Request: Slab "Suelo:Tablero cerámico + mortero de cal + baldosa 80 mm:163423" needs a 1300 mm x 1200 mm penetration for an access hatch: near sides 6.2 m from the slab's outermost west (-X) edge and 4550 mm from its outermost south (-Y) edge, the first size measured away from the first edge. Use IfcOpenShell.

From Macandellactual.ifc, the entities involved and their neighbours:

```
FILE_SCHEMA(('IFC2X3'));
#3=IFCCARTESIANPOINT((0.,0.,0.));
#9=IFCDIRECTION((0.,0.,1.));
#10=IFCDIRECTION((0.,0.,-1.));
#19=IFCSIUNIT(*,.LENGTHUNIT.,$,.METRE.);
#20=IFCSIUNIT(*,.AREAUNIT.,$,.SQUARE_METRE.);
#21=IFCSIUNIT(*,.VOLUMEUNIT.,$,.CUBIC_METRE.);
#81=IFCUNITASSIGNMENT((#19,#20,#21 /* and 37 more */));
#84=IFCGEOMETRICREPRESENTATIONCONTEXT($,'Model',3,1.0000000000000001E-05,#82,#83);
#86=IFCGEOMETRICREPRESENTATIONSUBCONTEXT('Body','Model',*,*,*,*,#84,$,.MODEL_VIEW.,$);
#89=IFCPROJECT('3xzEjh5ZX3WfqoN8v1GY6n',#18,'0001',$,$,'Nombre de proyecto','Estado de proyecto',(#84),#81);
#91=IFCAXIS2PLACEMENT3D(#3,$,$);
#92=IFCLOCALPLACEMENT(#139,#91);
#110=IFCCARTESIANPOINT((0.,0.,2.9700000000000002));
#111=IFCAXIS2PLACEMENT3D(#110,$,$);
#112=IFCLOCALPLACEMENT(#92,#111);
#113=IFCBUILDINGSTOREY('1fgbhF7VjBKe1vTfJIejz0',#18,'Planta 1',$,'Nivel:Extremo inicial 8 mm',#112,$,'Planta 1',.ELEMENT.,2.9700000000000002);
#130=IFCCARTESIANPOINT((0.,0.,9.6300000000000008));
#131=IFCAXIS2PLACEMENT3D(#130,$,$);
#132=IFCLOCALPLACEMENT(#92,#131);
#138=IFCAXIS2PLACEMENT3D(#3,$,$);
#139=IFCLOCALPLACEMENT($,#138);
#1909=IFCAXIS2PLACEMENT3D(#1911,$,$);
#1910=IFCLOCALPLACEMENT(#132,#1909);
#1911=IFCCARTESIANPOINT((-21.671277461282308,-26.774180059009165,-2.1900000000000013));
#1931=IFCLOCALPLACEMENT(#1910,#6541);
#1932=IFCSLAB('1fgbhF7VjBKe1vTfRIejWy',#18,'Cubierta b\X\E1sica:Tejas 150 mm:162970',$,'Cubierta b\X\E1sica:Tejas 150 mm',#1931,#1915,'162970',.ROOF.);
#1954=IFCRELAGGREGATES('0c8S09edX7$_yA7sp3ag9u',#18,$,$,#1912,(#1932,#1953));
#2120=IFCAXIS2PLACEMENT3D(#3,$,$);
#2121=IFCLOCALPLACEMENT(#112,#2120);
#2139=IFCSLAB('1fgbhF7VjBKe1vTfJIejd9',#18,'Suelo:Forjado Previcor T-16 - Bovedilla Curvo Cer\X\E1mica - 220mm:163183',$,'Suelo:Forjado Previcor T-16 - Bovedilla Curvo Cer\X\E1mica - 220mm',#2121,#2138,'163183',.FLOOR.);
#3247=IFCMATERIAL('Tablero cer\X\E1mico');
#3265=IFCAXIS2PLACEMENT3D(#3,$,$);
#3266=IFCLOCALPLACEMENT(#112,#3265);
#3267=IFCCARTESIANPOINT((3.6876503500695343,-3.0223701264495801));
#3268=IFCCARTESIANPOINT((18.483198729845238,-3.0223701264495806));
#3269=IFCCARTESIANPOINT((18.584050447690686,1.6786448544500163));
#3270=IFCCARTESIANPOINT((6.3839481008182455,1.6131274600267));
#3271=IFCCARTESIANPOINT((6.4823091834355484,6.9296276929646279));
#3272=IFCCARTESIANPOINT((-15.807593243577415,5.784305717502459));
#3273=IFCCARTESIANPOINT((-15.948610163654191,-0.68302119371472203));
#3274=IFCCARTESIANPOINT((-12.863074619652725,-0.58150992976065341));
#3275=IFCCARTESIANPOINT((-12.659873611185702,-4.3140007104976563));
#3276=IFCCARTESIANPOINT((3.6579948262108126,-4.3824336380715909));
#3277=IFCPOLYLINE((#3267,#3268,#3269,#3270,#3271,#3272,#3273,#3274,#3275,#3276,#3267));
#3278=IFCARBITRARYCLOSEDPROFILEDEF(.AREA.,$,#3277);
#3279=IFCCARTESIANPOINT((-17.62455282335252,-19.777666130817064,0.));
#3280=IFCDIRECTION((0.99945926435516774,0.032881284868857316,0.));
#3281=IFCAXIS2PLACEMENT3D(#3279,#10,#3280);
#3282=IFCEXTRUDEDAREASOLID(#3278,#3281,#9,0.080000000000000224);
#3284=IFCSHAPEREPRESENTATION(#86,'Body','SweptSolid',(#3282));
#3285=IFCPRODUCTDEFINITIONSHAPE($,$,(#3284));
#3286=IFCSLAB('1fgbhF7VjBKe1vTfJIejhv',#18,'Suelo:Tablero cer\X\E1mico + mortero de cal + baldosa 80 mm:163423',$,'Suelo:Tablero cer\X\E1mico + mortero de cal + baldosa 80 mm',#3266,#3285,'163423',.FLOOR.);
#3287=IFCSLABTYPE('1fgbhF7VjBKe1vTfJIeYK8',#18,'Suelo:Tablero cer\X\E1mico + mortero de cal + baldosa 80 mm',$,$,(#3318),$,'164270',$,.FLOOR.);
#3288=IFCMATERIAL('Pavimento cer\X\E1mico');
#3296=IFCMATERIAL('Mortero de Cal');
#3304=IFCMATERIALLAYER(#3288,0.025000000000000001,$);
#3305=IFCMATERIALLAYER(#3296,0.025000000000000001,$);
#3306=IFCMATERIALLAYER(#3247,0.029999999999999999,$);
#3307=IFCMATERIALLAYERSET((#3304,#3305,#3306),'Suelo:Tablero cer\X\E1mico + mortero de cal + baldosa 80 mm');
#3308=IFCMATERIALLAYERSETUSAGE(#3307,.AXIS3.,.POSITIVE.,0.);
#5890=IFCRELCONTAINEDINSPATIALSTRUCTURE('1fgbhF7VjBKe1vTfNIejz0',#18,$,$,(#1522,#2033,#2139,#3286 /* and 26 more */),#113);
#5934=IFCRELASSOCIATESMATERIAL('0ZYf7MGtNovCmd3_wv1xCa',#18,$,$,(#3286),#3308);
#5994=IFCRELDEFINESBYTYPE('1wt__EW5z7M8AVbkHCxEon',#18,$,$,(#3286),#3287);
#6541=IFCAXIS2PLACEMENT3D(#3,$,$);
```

```python
import numpy as np
import ifcopenshell
import ifcopenshell.api.feature
import ifcopenshell.api.geometry
import ifcopenshell.api.root
import ifcopenshell.geom
import ifcopenshell.util.placement
import ifcopenshell.util.representation
import ifcopenshell.util.shape
import ifcopenshell.util.unit

model = ifcopenshell.open("Macandellactual.ifc")
unit_scale = ifcopenshell.util.unit.calculate_unit_scale(model)
settings = ifcopenshell.geom.settings()


def volume(element):
    """Net volume in cubic metres, openings subtracted."""
    shape = ifcopenshell.geom.create_shape(settings, element)
    return ifcopenshell.util.shape.get_volume(shape.geometry)


slab = model.by_id(3286)
before = volume(slab)

# Extent in the slab's own axes, in metres. The edges named are its -X and -Y sides.
slab_shape = ifcopenshell.geom.create_shape(settings, slab)
vertices = ifcopenshell.util.shape.get_vertices(slab_shape.geometry)
x_min, y_min, bottom = vertices.min(axis=0)
top = vertices[:, 2].max()

opening = ifcopenshell.api.root.create_entity(model, ifc_class="IfcOpeningElement", name="Access hatch opening")
context = ifcopenshell.util.representation.get_context(model, "Model", "Body", "MODEL_VIEW")
width, depth = 1.3, 1.2
outline = [(0.0, 0.0), (width, 0.0), (width, depth), (0.0, depth), (0.0, 0.0)]
# Overshoot both faces by 50 mm so the cut is clean.
shape = ifcopenshell.api.geometry.add_slab_representation(
    model, context=context, depth=top - bottom + 0.1, polyline=outline
)
ifcopenshell.api.geometry.assign_representation(model, product=opening, representation=shape)

matrix = ifcopenshell.util.placement.get_local_placement(slab.ObjectPlacement)
matrix[:, 3] = matrix @ np.append(np.array([x_min + 6.2, y_min + 4.55, bottom - 0.05]) / unit_scale, 1.0)
ifcopenshell.api.geometry.edit_object_placement(model, product=opening, matrix=matrix, is_si=False)
ifcopenshell.api.feature.add_feature(model, feature=opening, element=slab)

after = volume(slab)

print(f"slab volume {before:.3f} -> {after:.3f} m3")

model.write("Macandellactual-out.ifc")
```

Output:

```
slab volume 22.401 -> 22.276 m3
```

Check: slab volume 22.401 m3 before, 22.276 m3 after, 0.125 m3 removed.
